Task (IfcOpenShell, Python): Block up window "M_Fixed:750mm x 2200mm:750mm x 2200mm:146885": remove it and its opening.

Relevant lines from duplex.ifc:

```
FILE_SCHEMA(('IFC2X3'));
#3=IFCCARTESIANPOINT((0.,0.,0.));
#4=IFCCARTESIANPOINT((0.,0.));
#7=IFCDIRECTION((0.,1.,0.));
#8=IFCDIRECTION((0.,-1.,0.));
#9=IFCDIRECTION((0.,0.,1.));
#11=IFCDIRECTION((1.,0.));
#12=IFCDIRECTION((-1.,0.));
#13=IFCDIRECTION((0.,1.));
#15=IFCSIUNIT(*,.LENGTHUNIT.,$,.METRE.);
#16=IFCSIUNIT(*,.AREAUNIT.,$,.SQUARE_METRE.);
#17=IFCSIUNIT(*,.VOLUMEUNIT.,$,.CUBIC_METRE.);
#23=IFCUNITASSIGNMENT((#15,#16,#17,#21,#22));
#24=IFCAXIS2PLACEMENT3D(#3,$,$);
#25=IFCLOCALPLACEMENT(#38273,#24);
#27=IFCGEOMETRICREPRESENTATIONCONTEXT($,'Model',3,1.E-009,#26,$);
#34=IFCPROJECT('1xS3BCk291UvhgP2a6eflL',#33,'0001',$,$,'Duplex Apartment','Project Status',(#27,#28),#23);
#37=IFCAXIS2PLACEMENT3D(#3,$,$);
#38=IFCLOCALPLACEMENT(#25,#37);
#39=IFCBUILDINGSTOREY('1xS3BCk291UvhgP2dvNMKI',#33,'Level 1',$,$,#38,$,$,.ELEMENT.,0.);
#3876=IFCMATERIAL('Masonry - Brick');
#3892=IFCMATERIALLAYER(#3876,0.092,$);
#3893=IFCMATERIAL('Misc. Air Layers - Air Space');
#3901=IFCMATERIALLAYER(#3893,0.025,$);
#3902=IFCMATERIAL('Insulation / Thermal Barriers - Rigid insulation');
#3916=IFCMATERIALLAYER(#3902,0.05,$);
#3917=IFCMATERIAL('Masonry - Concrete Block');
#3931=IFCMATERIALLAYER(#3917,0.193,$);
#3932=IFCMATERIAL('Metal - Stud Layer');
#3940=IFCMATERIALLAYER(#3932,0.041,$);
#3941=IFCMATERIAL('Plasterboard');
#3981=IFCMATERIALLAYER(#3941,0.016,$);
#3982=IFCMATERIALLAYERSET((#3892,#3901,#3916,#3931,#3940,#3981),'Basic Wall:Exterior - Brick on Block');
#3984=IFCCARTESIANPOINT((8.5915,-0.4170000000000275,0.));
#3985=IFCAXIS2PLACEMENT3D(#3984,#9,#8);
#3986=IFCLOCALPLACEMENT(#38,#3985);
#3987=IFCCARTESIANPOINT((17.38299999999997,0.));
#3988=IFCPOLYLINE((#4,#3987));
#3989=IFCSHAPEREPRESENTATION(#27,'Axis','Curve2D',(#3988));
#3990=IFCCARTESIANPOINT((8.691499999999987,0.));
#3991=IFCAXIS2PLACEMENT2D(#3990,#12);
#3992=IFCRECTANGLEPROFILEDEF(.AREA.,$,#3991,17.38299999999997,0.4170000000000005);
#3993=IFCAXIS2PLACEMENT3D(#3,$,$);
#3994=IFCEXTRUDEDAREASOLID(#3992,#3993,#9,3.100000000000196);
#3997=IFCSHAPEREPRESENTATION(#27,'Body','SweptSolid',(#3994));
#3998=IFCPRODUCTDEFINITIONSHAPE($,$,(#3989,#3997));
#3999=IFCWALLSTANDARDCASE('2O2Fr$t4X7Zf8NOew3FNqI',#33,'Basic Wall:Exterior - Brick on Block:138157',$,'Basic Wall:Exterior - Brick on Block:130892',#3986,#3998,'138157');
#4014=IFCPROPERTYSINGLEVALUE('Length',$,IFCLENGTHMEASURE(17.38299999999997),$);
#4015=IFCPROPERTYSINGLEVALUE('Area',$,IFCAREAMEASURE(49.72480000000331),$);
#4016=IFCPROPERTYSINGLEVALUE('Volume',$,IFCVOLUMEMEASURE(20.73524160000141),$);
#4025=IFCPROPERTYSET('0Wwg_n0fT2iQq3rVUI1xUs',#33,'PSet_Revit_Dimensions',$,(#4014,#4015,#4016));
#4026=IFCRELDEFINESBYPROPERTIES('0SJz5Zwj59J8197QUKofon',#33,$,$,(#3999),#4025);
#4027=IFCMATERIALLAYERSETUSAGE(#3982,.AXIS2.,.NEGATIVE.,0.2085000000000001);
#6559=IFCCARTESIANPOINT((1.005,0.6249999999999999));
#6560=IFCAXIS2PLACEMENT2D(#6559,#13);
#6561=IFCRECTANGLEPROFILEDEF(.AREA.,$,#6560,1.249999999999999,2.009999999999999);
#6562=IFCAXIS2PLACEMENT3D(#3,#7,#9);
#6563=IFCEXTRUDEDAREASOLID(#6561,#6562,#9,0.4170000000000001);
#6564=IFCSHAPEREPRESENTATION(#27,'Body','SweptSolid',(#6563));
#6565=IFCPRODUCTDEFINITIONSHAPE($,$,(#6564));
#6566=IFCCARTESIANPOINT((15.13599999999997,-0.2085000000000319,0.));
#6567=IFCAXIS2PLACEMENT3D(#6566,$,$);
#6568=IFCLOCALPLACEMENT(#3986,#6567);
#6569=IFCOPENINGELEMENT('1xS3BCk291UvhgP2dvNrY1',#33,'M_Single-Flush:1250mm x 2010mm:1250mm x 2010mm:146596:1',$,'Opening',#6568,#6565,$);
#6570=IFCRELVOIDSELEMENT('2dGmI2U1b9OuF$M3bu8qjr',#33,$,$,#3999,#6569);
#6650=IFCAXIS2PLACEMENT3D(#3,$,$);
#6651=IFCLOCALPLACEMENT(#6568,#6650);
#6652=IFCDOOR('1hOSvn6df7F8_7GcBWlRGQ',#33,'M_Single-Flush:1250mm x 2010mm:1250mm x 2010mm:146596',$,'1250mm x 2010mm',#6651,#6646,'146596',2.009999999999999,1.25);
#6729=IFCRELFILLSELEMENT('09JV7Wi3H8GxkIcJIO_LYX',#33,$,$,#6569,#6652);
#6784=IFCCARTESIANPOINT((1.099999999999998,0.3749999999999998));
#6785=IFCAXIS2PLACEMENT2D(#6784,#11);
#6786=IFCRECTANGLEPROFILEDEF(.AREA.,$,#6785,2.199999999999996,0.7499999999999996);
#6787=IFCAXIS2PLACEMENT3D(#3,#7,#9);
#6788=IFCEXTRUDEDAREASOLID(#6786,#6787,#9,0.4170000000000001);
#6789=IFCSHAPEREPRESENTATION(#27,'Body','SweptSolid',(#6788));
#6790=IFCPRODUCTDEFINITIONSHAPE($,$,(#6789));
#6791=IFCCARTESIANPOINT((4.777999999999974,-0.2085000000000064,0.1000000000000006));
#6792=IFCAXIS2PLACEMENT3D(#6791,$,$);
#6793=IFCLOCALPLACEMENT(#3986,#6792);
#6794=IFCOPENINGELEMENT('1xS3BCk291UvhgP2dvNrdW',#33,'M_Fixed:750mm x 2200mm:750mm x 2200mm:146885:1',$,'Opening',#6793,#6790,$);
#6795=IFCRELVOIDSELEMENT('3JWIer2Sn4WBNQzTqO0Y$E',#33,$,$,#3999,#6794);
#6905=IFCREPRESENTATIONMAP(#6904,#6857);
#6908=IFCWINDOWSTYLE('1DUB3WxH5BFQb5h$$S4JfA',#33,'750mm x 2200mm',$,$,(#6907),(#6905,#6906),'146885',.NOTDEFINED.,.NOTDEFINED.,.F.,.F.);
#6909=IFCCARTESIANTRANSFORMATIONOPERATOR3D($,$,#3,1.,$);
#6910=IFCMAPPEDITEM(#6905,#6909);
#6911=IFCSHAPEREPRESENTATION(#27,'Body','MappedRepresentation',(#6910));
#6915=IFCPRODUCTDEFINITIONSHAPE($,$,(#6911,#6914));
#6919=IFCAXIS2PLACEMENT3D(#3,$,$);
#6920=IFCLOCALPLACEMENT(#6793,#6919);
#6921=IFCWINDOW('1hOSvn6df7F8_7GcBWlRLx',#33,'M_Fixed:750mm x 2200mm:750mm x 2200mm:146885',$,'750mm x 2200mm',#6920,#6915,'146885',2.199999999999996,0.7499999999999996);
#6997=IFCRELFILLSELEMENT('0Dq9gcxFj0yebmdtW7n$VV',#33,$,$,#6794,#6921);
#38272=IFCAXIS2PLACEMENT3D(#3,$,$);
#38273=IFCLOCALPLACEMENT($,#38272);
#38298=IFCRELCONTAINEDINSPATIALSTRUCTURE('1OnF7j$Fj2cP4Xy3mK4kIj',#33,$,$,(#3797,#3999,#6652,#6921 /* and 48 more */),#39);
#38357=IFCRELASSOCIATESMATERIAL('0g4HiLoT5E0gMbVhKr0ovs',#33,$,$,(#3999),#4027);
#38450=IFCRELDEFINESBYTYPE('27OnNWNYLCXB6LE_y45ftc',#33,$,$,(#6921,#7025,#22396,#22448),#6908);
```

```python
import ifcopenshell
import ifcopenshell.api.feature
import ifcopenshell.api.pset
import ifcopenshell.api.root
import ifcopenshell.geom
import ifcopenshell.util.element
import ifcopenshell.util.shape
import ifcopenshell.util.unit

model = ifcopenshell.open("duplex.ifc")
area_scale = ifcopenshell.util.unit.calculate_unit_scale(model, "AREAUNIT")
volume_scale = ifcopenshell.util.unit.calculate_unit_scale(model, "VOLUMEUNIT")
settings = ifcopenshell.geom.settings()


def volume(element):
    """Net volume in cubic metres, openings subtracted."""
    shape = ifcopenshell.geom.create_shape(settings, element)
    return ifcopenshell.util.shape.get_volume(shape.geometry)


window = model.by_id(6921)
opening = window.FillsVoids[0].RelatingOpeningElement
wall = opening.VoidsElements[0].RelatingBuildingElement
before = volume(wall)

ifcopenshell.api.root.remove_product(model, product=window)
ifcopenshell.api.feature.remove_feature(model, feature=opening)

after = volume(wall)
thickness = 0.417  # wall thickness in metres

# Update the wall's stored quantities.
pset = model.by_id(ifcopenshell.util.element.get_pset(wall, "PSet_Revit_Dimensions", should_inherit=False)["id"])
ifcopenshell.api.pset.edit_pset(model, pset=pset, properties={
    "Area": model.create_entity("IfcAreaMeasure", after / thickness / area_scale),
    "Volume": model.create_entity("IfcVolumeMeasure", after / volume_scale),
})

print(f"wall volume {before:.3f} -> {after:.3f} m3")

model.write("duplex_updated.ifc")
```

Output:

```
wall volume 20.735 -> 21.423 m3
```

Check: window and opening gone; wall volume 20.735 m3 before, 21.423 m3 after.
